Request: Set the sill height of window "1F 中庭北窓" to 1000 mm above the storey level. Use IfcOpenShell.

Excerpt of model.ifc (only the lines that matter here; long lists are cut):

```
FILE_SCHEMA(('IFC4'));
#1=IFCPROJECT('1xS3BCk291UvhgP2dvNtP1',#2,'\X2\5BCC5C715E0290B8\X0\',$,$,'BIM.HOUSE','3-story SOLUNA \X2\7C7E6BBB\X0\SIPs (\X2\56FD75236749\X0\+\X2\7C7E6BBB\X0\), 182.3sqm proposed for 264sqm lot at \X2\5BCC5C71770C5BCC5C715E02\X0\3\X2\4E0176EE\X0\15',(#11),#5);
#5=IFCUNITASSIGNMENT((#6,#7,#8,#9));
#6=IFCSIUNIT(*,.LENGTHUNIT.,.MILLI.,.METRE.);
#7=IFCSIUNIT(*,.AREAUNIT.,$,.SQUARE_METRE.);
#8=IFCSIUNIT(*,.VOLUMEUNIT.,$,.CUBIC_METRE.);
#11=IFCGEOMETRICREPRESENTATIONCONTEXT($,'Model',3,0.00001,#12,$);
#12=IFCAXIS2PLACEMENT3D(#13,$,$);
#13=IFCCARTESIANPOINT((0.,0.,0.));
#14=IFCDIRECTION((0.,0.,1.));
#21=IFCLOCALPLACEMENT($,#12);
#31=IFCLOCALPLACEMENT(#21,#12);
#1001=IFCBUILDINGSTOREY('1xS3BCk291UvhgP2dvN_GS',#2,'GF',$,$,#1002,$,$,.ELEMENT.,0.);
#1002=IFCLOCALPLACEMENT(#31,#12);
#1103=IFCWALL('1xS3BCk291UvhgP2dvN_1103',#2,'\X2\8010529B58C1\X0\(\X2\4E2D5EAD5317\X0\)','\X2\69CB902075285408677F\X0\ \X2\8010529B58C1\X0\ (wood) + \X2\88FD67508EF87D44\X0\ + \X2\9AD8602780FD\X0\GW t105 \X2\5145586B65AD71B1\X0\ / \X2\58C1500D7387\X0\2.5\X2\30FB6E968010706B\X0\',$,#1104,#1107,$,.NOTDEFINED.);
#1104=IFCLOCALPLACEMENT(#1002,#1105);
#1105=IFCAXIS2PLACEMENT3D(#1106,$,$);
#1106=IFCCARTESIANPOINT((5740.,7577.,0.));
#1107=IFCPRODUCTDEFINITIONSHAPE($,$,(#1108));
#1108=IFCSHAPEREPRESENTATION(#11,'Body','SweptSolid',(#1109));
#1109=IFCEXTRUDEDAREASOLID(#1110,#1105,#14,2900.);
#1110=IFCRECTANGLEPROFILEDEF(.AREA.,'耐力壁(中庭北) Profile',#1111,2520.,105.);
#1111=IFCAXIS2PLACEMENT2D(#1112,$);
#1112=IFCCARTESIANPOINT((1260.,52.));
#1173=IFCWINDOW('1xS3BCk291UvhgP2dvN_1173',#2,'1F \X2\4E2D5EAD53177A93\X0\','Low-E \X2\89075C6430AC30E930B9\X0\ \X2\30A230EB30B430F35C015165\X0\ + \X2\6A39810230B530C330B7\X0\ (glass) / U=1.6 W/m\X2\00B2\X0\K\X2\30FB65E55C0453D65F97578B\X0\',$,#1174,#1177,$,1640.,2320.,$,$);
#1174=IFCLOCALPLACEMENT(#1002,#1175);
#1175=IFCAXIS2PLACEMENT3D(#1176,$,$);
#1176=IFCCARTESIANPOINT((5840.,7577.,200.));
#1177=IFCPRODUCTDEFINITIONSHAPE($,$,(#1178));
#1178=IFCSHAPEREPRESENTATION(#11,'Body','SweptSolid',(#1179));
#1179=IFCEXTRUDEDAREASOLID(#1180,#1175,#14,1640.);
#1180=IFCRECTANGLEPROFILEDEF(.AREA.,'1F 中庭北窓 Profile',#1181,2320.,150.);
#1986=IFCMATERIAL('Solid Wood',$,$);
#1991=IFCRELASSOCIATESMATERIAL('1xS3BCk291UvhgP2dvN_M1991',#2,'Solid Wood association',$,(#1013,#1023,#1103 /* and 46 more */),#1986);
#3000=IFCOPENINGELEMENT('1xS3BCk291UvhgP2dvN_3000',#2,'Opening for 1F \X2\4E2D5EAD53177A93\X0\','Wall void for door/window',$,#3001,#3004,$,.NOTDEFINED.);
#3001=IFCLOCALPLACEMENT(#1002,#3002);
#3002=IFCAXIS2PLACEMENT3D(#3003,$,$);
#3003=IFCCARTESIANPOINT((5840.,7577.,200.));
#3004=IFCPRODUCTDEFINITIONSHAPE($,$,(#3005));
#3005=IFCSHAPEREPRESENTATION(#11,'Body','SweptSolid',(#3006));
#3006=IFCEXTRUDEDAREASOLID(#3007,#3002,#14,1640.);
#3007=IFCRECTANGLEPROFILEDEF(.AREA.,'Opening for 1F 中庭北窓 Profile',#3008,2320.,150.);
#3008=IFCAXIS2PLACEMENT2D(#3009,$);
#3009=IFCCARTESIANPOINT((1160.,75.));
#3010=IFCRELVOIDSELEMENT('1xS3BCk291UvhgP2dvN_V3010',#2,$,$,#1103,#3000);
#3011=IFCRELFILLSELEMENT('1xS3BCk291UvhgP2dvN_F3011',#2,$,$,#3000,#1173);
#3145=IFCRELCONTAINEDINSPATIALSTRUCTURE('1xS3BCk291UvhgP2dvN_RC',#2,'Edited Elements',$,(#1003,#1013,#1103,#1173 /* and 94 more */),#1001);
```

```python
import numpy as np
import ifcopenshell
import ifcopenshell.api.geometry
import ifcopenshell.geom
import ifcopenshell.util.element
import ifcopenshell.util.placement
import ifcopenshell.util.shape
import ifcopenshell.util.unit

model = ifcopenshell.open("model.ifc")
unit_scale = ifcopenshell.util.unit.calculate_unit_scale(model)

window = model.by_guid("1xS3BCk291UvhgP2dvN_1173")
opening = window.FillsVoids[0].RelatingOpeningElement
storey = ifcopenshell.util.element.get_container(window, ifc_class="IfcBuildingStorey")
level = ifcopenshell.util.placement.get_local_placement(storey.ObjectPlacement)[2, 3]

# The opening's origin need not be at the sill, so measure its lowest point.
shape = ifcopenshell.geom.create_shape(ifcopenshell.geom.settings(), opening)
bottom = ifcopenshell.util.shape.get_shape_bottom_elevation(shape, shape.geometry) / unit_scale
dz = level + 1000.0 - bottom

shift = np.array([0.0, 0.0, dz])
# The window is not placed relative to its opening, so move both.
for product in (opening, window):
    matrix = ifcopenshell.util.placement.get_local_placement(product.ObjectPlacement)
    matrix[:3, 3] += shift
    ifcopenshell.api.geometry.edit_object_placement(model, product=product, matrix=matrix, is_si=False)

print(f"moved by {dz * unit_scale:+.3f} m")

model.write("model_updated.ifc")
```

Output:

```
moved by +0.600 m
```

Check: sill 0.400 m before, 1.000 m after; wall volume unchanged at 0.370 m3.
